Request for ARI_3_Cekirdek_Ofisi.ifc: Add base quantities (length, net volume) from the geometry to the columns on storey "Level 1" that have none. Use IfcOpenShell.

First a look at what the model holds.

```python
import ifcopenshell
import ifcopenshell.util.element
import ifcopenshell.util.unit

model = ifcopenshell.open("ARI_3_Cekirdek_Ofisi.ifc")
print(model.schema)
for unit_type in ("LENGTHUNIT", "AREAUNIT", "VOLUMEUNIT"):
    print(unit_type, ifcopenshell.util.unit.calculate_unit_scale(model, unit_type))
storey = next(s for s in model.by_type("IfcBuildingStorey") if s.Name == "Level 1")
columns = [e for e in ifcopenshell.util.element.get_decomposition(storey) if e.is_a("IfcColumn")]
for e in sorted(columns, key=lambda e: e.id()):
    print(e.id(), e.is_a(), e.Name, list(ifcopenshell.util.element.get_psets(e, qtos_only=True)), sep=" | ")
```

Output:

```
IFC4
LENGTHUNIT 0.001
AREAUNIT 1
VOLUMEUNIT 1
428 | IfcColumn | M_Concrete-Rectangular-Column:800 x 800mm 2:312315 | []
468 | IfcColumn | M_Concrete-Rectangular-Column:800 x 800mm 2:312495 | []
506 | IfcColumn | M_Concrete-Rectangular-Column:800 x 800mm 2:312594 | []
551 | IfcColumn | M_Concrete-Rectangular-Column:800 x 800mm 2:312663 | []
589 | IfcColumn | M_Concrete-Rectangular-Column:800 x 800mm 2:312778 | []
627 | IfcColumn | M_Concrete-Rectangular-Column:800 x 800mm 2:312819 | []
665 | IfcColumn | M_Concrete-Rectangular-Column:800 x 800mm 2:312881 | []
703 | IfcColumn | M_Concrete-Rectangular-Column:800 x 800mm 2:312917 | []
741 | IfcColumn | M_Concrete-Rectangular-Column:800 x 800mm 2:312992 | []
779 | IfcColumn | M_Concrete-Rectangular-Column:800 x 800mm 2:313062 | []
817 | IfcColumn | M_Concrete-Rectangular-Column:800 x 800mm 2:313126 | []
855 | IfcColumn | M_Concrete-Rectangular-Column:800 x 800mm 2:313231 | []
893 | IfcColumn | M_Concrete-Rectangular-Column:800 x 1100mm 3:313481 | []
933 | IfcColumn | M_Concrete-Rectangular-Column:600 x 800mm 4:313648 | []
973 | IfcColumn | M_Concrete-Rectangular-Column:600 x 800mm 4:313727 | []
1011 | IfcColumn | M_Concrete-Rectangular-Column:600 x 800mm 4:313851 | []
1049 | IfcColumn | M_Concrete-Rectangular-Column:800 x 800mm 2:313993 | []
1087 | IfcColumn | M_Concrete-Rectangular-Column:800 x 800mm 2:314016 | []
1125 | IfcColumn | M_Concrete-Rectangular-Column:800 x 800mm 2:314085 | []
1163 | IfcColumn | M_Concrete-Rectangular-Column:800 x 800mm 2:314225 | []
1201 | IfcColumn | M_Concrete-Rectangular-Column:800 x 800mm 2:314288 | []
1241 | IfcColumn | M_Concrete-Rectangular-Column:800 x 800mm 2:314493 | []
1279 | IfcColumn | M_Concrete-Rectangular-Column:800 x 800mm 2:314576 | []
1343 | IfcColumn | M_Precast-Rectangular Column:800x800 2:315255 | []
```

```python
import ifcopenshell
import ifcopenshell.api.pset
import ifcopenshell.geom
import ifcopenshell.util.element
import ifcopenshell.util.shape
import ifcopenshell.util.unit

model = ifcopenshell.open("ARI_3_Cekirdek_Ofisi.ifc")
unit_scale = ifcopenshell.util.unit.calculate_unit_scale(model)
volume_scale = ifcopenshell.util.unit.calculate_unit_scale(model, "VOLUMEUNIT")
settings = ifcopenshell.geom.settings()

storey = next(s for s in model.by_type("IfcBuildingStorey") if s.Name == "Level 1")
columns = [e for e in ifcopenshell.util.element.get_decomposition(storey) if e.is_a("IfcColumn")]

for e in sorted(columns, key=lambda e: e.id()):
    if ifcopenshell.util.element.get_psets(e, qtos_only=True, should_inherit=False):
        continue
    # Geometry comes back in metres, in the element's own axes.
    shape = ifcopenshell.geom.create_shape(settings, e)
    values = {
        "Length": ifcopenshell.util.shape.get_z(shape.geometry) / unit_scale,
        "NetVolume": ifcopenshell.util.shape.get_volume(shape.geometry) / volume_scale,
    }
    qto = ifcopenshell.api.pset.add_qto(model, product=e, name="Qto_ColumnBaseQuantities")
    ifcopenshell.api.pset.edit_qto(model, qto=qto, properties=values)
    print(e.id(), {k: round(v, 3) for k, v in values.items()})

model.write("ARI_3_Cekirdek_Ofisi-out.ifc")
```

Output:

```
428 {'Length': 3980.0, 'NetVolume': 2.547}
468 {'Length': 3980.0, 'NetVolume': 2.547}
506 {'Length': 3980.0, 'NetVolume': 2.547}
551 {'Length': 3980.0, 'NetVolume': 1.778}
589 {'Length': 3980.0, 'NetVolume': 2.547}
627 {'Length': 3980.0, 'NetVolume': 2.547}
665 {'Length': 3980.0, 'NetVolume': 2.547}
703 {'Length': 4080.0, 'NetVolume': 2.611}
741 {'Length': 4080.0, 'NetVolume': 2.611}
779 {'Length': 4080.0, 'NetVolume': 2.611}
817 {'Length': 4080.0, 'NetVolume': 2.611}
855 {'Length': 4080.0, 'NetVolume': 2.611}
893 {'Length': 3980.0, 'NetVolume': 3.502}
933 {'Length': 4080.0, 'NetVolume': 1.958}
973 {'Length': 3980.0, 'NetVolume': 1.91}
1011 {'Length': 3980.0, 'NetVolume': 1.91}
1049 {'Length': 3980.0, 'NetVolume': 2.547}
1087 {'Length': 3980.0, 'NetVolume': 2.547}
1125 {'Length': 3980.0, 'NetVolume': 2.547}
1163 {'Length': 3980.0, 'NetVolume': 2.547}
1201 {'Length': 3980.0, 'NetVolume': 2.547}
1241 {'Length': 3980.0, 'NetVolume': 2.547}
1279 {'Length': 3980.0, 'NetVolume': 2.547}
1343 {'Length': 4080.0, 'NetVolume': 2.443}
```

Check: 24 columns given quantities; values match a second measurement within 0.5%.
